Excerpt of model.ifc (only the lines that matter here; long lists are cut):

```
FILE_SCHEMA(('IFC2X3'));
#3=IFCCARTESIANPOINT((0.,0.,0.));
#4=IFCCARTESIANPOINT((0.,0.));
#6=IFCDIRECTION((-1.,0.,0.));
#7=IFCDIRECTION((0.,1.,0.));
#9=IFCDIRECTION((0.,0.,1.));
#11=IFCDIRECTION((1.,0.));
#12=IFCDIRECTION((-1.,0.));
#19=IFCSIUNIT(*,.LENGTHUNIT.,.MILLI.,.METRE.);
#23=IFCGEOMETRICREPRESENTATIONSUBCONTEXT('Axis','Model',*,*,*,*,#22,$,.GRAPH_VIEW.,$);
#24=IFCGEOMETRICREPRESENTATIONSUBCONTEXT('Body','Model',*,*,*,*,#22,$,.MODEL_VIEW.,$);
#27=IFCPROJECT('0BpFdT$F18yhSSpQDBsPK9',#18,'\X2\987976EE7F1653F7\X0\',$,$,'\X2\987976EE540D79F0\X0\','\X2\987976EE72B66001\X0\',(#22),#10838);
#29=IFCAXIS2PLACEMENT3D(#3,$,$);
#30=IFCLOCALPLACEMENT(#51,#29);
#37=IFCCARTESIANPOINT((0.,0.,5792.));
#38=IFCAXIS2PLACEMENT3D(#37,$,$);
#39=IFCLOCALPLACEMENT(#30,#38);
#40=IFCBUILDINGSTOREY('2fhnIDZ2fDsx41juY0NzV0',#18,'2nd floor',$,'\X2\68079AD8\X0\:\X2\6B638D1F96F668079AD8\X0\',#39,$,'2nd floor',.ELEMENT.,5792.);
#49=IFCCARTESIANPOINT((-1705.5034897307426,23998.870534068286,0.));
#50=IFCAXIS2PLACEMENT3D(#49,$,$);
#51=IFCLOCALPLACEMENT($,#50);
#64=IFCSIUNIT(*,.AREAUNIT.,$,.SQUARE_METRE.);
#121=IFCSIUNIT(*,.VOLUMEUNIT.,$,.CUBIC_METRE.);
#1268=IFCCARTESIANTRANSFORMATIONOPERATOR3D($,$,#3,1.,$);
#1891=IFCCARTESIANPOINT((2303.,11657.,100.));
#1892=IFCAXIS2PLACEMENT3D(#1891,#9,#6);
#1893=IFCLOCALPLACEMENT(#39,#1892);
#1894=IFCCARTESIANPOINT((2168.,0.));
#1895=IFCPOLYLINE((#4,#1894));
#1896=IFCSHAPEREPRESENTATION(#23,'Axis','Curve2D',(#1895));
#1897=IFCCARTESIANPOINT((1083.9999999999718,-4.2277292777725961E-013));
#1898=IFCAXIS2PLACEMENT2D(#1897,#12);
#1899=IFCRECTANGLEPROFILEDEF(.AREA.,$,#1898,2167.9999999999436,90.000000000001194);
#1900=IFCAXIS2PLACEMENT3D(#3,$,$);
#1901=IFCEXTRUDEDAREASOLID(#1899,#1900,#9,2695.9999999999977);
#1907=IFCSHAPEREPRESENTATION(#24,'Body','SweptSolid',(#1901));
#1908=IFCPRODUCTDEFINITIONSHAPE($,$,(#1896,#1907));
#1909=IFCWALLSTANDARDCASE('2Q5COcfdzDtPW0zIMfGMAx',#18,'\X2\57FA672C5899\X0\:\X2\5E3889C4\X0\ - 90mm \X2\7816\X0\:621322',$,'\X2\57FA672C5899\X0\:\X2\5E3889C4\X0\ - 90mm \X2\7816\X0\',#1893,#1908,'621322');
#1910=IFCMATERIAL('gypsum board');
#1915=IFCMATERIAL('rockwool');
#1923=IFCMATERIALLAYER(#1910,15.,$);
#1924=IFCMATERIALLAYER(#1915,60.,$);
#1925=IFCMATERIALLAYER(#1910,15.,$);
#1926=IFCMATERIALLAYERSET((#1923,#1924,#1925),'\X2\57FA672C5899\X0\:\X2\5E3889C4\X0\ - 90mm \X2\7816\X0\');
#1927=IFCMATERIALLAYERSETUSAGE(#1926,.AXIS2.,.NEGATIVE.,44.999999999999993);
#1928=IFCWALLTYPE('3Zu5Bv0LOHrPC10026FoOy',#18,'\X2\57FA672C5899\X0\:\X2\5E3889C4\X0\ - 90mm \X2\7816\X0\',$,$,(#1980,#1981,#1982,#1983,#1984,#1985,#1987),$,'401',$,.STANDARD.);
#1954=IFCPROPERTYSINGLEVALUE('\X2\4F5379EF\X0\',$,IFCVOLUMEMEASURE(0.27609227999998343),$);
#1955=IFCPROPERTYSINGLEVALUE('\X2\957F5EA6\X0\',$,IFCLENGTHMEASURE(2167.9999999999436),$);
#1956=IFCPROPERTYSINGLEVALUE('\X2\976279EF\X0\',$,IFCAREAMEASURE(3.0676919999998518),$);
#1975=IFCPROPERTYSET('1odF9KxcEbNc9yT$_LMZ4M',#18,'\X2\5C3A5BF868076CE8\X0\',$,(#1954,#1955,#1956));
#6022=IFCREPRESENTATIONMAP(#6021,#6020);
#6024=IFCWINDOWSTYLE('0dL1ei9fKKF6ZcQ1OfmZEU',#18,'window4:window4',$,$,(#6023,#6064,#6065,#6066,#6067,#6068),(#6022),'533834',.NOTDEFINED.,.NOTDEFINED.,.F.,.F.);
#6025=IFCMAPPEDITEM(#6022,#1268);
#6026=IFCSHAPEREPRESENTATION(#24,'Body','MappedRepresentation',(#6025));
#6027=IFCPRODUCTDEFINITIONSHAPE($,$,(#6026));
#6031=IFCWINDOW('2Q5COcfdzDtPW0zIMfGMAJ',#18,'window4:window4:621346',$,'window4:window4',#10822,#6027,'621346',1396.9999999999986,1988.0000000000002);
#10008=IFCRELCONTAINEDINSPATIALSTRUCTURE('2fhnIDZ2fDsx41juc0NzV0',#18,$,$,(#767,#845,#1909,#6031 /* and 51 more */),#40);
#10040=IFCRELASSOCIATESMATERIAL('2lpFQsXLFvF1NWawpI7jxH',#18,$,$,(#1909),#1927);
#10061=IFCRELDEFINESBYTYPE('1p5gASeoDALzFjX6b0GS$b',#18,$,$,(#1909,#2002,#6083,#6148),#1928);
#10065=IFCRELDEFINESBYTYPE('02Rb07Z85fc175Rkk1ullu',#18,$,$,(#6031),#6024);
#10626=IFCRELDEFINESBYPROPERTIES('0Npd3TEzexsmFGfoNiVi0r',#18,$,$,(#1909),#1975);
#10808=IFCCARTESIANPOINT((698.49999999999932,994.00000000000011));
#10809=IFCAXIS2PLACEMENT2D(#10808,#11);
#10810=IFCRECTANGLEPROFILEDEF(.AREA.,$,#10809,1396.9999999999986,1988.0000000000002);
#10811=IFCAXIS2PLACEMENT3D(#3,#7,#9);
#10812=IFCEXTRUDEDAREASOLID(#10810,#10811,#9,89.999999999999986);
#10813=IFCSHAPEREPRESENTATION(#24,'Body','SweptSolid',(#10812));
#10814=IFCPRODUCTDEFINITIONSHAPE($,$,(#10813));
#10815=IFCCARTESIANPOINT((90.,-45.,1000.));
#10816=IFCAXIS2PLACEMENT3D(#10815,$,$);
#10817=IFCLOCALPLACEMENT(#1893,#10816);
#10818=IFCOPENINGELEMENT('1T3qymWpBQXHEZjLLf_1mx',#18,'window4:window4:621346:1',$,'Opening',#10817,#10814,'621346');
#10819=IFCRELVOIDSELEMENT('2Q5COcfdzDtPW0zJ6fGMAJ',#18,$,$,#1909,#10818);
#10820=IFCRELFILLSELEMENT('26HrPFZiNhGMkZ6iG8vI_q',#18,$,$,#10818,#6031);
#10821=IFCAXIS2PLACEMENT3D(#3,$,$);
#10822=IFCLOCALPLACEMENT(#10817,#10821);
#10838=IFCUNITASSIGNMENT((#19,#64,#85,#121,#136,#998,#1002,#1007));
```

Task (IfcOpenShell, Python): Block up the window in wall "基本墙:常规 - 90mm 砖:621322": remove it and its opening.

```python
import ifcopenshell
import ifcopenshell.api.feature
import ifcopenshell.api.pset
import ifcopenshell.api.root
import ifcopenshell.geom
import ifcopenshell.util.element
import ifcopenshell.util.shape
import ifcopenshell.util.unit

model = ifcopenshell.open("model.ifc")
area_scale = ifcopenshell.util.unit.calculate_unit_scale(model, "AREAUNIT")
volume_scale = ifcopenshell.util.unit.calculate_unit_scale(model, "VOLUMEUNIT")
settings = ifcopenshell.geom.settings()


def volume(element):
    """Net volume in cubic metres, openings subtracted."""
    shape = ifcopenshell.geom.create_shape(settings, element)
    return ifcopenshell.util.shape.get_volume(shape.geometry)


window = model.by_guid("2Q5COcfdzDtPW0zIMfGMAJ")
opening = window.FillsVoids[0].RelatingOpeningElement
wall = opening.VoidsElements[0].RelatingBuildingElement
before = volume(wall)

ifcopenshell.api.root.remove_product(model, product=window)
ifcopenshell.api.feature.remove_feature(model, feature=opening)

after = volume(wall)
thickness = 0.09  # wall thickness in metres

# Update the wall's stored quantities.
pset = model.by_id(ifcopenshell.util.element.get_pset(wall, "尺寸标注", should_inherit=False)["id"])
ifcopenshell.api.pset.edit_pset(model, pset=pset, properties={
    "体积": model.create_entity("IfcVolumeMeasure", after / volume_scale),
    "面积": model.create_entity("IfcAreaMeasure", after / thickness / area_scale),
})

print(f"wall volume {before:.3f} -> {after:.3f} m3")

model.write("model_edited.ifc")
```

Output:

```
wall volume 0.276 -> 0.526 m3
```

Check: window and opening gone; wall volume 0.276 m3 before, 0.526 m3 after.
